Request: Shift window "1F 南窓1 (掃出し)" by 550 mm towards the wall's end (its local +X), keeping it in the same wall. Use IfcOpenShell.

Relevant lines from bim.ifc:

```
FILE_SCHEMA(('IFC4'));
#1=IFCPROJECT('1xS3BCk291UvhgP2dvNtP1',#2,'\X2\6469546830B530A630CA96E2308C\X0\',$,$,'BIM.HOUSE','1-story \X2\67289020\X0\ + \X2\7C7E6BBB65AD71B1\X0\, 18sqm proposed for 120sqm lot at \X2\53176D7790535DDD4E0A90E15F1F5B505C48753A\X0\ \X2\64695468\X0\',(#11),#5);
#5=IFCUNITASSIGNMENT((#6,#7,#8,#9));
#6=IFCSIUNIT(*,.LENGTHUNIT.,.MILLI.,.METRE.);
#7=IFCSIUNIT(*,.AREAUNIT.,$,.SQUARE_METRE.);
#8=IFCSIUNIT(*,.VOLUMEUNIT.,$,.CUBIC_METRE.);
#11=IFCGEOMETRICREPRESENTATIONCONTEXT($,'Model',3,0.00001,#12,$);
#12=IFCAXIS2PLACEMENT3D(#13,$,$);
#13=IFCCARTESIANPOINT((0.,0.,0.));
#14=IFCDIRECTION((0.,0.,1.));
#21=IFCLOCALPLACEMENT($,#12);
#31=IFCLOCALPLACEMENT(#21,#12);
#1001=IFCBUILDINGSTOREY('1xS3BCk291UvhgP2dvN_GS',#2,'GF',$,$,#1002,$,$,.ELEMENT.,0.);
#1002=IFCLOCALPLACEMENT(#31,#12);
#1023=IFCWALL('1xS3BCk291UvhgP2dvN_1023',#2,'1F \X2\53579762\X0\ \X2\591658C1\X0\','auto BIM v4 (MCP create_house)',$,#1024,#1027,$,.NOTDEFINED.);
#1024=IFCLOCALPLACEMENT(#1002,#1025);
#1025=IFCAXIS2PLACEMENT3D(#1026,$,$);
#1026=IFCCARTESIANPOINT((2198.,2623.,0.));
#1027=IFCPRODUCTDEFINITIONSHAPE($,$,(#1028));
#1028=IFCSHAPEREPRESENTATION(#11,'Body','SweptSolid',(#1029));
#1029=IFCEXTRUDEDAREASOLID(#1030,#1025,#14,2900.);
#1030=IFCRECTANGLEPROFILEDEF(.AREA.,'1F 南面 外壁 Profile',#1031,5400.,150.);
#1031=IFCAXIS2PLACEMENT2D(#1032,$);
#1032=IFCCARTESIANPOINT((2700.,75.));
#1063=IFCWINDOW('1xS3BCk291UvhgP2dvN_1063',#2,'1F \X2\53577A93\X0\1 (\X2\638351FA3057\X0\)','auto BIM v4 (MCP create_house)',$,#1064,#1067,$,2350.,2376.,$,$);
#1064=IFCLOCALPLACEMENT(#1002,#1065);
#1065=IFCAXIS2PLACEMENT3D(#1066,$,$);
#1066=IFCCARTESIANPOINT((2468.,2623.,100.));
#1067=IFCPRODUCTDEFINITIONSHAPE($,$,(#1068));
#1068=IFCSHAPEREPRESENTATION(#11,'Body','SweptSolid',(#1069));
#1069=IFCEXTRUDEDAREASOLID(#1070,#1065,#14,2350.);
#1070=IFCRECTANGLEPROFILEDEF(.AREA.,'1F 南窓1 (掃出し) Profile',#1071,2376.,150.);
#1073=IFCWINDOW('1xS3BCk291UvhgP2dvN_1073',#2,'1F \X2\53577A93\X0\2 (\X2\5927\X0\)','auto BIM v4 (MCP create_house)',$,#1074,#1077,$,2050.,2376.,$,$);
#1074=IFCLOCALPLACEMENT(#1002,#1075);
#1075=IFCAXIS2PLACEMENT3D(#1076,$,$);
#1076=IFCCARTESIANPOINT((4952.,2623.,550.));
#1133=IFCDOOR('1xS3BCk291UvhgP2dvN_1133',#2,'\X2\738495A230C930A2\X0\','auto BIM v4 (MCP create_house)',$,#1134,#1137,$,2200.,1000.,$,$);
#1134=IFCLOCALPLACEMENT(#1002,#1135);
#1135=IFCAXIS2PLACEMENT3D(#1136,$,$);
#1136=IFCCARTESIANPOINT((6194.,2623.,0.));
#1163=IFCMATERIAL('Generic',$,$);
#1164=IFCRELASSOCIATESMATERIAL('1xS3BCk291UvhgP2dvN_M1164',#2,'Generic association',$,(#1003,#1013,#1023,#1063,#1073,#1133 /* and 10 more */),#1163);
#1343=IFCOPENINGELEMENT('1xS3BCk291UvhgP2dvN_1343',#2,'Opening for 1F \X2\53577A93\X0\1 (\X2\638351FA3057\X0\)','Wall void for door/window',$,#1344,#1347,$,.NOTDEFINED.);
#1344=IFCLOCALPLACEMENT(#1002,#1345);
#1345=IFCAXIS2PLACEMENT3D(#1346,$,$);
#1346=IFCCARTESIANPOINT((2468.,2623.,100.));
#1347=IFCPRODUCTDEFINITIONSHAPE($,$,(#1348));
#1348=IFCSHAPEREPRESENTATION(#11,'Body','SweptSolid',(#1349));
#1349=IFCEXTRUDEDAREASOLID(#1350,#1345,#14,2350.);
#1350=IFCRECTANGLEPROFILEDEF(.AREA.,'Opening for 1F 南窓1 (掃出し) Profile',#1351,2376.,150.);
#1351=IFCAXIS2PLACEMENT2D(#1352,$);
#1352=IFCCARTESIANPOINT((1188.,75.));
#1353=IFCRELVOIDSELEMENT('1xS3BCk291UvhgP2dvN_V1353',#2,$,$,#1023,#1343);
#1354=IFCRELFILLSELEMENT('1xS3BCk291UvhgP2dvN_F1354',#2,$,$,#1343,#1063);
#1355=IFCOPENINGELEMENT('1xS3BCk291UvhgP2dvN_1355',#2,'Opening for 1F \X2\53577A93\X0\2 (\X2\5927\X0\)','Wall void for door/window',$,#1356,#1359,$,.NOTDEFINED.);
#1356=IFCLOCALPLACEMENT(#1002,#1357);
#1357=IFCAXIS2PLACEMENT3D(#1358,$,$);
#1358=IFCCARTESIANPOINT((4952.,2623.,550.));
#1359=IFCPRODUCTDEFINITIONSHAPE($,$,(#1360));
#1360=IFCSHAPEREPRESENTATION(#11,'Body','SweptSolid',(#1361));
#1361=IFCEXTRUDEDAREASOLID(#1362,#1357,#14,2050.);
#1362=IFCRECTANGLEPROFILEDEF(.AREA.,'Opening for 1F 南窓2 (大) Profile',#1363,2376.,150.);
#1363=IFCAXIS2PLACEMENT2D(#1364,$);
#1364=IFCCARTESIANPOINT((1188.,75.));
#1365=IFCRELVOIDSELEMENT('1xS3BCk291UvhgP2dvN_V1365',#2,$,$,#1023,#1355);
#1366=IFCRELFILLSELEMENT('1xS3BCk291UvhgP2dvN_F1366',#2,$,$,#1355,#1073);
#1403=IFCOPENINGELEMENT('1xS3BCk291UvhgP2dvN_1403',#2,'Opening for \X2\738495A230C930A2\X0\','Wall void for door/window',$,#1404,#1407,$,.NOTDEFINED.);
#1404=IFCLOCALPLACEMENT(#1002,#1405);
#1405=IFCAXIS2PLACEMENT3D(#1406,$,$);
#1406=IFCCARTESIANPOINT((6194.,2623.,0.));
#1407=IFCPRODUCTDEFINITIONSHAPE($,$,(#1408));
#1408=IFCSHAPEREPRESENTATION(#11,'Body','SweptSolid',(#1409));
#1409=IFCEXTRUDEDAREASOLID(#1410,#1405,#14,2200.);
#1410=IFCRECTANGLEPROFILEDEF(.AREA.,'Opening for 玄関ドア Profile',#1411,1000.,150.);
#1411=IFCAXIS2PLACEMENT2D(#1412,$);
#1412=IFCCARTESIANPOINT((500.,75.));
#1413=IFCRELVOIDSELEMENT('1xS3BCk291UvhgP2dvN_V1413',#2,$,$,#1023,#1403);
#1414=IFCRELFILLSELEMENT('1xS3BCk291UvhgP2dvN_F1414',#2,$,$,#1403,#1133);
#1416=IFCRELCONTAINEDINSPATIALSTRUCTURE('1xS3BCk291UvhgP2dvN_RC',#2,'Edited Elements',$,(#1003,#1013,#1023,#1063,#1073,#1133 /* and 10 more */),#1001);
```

```python
import ifcopenshell
import ifcopenshell.api.geometry
import ifcopenshell.util.placement
import ifcopenshell.util.unit

model = ifcopenshell.open("bim.ifc")
unit_scale = ifcopenshell.util.unit.calculate_unit_scale(model)

window = model.by_id(1063)
opening = window.FillsVoids[0].RelatingOpeningElement
wall = opening.VoidsElements[0].RelatingBuildingElement

wall_matrix = ifcopenshell.util.placement.get_local_placement(wall.ObjectPlacement)
shift = wall_matrix[:3, 0] * 0.55 / unit_scale
before = ifcopenshell.util.placement.get_local_placement(window.ObjectPlacement)[:3, 3].copy()

# The window is not placed relative to its opening, so move both.
for product in (opening, window):
    matrix = ifcopenshell.util.placement.get_local_placement(product.ObjectPlacement)
    matrix[:3, 3] += shift
    ifcopenshell.api.geometry.edit_object_placement(model, product=product, matrix=matrix, is_si=False)

after = ifcopenshell.util.placement.get_local_placement(window.ObjectPlacement)[:3, 3]
print("window moved by", (after - before).round(3) + 0.0)

model.write("bim_rev.ifc")
```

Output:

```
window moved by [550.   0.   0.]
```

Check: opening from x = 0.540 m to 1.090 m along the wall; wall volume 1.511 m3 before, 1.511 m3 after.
